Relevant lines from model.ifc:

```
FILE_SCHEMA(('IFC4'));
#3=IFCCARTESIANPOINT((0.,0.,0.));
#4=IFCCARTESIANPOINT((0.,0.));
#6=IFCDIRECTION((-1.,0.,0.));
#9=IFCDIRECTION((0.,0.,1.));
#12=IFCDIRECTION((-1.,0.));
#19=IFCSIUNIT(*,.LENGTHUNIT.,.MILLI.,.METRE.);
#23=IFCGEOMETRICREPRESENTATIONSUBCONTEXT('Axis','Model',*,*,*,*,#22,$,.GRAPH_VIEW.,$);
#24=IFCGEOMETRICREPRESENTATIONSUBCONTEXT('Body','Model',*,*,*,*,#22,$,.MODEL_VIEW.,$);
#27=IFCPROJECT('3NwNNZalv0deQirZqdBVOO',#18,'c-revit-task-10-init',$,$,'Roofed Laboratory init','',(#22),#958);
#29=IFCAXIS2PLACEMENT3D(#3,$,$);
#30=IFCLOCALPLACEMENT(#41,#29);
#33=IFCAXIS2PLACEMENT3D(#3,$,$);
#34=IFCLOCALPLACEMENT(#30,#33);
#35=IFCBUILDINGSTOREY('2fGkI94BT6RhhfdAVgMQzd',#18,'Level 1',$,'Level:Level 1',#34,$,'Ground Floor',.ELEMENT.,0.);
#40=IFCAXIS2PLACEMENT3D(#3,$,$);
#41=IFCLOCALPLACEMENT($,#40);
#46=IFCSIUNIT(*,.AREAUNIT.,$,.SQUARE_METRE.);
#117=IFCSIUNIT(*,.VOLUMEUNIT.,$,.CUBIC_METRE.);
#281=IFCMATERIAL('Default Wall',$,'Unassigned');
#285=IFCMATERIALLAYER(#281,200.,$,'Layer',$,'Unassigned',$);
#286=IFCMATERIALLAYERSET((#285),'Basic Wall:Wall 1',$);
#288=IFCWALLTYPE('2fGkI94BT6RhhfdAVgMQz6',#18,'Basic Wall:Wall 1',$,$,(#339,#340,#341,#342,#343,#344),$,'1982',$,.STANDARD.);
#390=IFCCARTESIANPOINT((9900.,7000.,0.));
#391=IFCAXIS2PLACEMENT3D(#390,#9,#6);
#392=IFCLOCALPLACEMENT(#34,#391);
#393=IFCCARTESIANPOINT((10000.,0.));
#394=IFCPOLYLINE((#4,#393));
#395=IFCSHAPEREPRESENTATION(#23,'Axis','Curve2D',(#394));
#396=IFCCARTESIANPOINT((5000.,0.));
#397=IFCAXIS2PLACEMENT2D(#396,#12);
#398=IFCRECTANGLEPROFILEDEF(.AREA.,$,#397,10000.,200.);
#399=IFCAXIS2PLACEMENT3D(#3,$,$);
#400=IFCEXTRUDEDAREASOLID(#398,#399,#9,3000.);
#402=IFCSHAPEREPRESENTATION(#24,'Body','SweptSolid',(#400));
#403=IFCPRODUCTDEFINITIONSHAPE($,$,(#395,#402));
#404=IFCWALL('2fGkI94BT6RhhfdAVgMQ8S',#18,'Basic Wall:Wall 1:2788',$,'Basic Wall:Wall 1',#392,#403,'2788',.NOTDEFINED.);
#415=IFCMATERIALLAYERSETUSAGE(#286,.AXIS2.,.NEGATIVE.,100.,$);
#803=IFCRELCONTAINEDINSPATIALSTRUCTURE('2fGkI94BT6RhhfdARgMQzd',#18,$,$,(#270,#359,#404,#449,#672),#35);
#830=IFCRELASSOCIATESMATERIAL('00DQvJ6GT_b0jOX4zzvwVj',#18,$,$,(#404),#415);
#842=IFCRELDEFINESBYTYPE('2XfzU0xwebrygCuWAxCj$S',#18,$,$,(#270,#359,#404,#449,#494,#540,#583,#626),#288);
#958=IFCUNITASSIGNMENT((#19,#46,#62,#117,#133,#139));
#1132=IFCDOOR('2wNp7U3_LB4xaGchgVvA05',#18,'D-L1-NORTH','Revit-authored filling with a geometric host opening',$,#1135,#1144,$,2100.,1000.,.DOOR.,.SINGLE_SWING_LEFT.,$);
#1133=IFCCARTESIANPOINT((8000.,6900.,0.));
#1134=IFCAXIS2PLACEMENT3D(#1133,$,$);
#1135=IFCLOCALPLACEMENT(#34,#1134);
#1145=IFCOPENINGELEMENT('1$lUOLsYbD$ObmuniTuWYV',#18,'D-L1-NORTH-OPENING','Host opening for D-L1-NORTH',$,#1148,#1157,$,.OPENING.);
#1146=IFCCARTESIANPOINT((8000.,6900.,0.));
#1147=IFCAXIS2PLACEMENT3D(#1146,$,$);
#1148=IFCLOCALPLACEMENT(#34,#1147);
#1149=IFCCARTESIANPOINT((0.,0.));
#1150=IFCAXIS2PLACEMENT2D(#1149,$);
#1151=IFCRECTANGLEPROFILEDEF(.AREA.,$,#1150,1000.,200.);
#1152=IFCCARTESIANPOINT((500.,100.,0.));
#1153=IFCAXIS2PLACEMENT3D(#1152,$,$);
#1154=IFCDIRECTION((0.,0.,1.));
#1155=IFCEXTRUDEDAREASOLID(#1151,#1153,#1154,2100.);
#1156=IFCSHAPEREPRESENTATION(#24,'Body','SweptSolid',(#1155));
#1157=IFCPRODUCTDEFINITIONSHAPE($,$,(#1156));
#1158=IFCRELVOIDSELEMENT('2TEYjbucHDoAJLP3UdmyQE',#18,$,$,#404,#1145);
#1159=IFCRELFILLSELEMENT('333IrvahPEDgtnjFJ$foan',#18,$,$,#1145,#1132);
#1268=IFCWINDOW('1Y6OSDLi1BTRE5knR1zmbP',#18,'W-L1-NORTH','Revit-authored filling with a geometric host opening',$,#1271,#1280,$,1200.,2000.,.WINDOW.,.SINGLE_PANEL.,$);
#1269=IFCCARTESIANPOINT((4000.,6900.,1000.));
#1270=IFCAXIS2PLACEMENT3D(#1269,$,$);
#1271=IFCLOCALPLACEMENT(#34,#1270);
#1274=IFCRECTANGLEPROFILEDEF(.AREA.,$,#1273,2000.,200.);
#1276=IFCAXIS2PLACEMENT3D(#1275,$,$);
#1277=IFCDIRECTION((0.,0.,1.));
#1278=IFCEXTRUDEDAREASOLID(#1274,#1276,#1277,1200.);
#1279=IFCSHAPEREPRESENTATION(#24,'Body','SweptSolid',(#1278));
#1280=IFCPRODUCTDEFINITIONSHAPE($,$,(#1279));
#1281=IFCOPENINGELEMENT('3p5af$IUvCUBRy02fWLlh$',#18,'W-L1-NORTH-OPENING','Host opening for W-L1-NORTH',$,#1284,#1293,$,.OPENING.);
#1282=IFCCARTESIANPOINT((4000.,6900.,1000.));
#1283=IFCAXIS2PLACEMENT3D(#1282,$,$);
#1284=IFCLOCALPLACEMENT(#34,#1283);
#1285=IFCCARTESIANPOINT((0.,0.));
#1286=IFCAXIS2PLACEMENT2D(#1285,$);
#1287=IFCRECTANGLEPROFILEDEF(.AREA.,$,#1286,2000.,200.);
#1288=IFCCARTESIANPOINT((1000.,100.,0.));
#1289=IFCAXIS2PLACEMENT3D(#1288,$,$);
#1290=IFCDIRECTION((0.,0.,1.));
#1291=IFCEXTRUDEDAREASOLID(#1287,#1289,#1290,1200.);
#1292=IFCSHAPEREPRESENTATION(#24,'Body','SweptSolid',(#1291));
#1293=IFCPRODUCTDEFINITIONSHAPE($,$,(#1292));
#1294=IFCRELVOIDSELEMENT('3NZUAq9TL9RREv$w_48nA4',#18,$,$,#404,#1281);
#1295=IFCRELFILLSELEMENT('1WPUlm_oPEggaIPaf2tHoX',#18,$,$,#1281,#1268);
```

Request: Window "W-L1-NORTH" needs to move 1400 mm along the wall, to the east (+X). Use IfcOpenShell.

```python
import ifcopenshell
import ifcopenshell.api.geometry
import ifcopenshell.util.placement
import ifcopenshell.util.unit

model = ifcopenshell.open("model.ifc")
unit_scale = ifcopenshell.util.unit.calculate_unit_scale(model)

window = model.by_guid("1Y6OSDLi1BTRE5knR1zmbP")
opening = window.FillsVoids[0].RelatingOpeningElement
wall = opening.VoidsElements[0].RelatingBuildingElement

wall_matrix = ifcopenshell.util.placement.get_local_placement(wall.ObjectPlacement)
shift = wall_matrix[:3, 0] * -1.4 / unit_scale
before = ifcopenshell.util.placement.get_local_placement(window.ObjectPlacement)[:3, 3].copy()

# The window is not placed relative to its opening, so move both.
for product in (opening, window):
    matrix = ifcopenshell.util.placement.get_local_placement(product.ObjectPlacement)
    matrix[:3, 3] += shift
    ifcopenshell.api.geometry.edit_object_placement(model, product=product, matrix=matrix, is_si=False)

after = ifcopenshell.util.placement.get_local_placement(window.ObjectPlacement)[:3, 3]
print("window moved by", (after - before).round(3) + 0.0)

model.write("model-out.ifc")
```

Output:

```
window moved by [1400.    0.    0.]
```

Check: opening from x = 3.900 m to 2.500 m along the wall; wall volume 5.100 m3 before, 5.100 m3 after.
